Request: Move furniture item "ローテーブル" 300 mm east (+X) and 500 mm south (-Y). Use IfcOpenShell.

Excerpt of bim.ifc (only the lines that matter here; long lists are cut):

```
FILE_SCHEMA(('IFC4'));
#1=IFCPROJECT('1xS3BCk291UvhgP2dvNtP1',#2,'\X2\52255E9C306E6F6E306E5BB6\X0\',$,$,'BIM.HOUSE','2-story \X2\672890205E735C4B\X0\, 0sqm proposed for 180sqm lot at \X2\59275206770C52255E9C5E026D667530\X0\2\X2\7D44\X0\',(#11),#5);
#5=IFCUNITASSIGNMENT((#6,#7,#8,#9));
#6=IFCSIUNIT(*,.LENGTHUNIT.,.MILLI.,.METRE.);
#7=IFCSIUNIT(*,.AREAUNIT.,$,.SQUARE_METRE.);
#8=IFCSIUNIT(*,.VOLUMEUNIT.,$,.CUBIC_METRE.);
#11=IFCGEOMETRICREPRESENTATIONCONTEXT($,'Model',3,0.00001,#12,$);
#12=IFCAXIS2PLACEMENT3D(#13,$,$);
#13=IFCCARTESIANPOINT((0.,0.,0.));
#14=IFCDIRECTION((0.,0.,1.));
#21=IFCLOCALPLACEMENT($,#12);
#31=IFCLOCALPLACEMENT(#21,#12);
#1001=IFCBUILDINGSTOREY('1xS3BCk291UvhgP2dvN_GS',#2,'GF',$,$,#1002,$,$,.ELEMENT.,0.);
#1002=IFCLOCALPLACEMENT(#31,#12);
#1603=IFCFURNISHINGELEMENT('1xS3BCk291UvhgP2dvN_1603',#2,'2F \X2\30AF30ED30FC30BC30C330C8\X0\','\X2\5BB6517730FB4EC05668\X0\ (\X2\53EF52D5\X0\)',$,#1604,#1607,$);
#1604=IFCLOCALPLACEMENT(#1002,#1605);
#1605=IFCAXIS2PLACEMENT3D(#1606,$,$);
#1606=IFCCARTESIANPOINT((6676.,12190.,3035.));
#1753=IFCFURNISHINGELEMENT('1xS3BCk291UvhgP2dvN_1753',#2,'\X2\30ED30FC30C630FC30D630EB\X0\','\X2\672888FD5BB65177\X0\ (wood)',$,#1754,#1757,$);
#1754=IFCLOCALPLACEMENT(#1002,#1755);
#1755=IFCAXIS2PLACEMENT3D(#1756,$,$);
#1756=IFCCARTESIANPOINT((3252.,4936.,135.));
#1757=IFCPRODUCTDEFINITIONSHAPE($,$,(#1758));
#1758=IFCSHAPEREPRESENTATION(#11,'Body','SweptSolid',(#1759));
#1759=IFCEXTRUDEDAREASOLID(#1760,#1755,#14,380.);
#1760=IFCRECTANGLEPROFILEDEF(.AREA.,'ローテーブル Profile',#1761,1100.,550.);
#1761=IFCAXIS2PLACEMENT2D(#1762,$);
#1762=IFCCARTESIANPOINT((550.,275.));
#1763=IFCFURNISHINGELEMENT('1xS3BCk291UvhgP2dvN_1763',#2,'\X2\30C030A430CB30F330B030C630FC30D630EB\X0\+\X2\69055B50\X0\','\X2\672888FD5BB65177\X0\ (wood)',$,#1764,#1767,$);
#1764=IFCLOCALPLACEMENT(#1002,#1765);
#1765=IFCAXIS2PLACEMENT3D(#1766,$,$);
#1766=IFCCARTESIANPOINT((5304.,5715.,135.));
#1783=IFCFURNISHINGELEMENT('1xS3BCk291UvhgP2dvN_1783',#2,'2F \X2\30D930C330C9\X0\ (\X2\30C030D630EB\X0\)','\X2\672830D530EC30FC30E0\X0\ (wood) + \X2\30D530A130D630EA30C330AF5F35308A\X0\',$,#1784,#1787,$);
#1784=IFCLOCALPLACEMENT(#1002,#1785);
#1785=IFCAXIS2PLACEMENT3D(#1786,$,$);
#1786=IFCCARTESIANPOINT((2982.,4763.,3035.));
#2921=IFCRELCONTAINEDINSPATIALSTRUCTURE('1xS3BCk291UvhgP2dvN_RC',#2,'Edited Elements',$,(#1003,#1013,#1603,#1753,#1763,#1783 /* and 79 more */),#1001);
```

```python
import ifcopenshell
import ifcopenshell.api.geometry
import ifcopenshell.util.placement

model = ifcopenshell.open("bim.ifc")

item = model.by_guid("1xS3BCk291UvhgP2dvN_1753")
matrix = ifcopenshell.util.placement.get_local_placement(item.ObjectPlacement)
matrix[0, 3] += 300.0
matrix[1, 3] -= 500.0
ifcopenshell.api.geometry.edit_object_placement(model, product=item, matrix=matrix, is_si=False)

print(ifcopenshell.util.placement.get_local_placement(item.ObjectPlacement).round(3) + 0.0)

model.write("bim_edited.ifc")
```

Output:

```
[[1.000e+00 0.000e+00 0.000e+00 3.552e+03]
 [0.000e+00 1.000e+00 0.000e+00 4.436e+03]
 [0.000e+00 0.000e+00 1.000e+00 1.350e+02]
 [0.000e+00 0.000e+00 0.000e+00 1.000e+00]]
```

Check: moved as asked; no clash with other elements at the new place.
